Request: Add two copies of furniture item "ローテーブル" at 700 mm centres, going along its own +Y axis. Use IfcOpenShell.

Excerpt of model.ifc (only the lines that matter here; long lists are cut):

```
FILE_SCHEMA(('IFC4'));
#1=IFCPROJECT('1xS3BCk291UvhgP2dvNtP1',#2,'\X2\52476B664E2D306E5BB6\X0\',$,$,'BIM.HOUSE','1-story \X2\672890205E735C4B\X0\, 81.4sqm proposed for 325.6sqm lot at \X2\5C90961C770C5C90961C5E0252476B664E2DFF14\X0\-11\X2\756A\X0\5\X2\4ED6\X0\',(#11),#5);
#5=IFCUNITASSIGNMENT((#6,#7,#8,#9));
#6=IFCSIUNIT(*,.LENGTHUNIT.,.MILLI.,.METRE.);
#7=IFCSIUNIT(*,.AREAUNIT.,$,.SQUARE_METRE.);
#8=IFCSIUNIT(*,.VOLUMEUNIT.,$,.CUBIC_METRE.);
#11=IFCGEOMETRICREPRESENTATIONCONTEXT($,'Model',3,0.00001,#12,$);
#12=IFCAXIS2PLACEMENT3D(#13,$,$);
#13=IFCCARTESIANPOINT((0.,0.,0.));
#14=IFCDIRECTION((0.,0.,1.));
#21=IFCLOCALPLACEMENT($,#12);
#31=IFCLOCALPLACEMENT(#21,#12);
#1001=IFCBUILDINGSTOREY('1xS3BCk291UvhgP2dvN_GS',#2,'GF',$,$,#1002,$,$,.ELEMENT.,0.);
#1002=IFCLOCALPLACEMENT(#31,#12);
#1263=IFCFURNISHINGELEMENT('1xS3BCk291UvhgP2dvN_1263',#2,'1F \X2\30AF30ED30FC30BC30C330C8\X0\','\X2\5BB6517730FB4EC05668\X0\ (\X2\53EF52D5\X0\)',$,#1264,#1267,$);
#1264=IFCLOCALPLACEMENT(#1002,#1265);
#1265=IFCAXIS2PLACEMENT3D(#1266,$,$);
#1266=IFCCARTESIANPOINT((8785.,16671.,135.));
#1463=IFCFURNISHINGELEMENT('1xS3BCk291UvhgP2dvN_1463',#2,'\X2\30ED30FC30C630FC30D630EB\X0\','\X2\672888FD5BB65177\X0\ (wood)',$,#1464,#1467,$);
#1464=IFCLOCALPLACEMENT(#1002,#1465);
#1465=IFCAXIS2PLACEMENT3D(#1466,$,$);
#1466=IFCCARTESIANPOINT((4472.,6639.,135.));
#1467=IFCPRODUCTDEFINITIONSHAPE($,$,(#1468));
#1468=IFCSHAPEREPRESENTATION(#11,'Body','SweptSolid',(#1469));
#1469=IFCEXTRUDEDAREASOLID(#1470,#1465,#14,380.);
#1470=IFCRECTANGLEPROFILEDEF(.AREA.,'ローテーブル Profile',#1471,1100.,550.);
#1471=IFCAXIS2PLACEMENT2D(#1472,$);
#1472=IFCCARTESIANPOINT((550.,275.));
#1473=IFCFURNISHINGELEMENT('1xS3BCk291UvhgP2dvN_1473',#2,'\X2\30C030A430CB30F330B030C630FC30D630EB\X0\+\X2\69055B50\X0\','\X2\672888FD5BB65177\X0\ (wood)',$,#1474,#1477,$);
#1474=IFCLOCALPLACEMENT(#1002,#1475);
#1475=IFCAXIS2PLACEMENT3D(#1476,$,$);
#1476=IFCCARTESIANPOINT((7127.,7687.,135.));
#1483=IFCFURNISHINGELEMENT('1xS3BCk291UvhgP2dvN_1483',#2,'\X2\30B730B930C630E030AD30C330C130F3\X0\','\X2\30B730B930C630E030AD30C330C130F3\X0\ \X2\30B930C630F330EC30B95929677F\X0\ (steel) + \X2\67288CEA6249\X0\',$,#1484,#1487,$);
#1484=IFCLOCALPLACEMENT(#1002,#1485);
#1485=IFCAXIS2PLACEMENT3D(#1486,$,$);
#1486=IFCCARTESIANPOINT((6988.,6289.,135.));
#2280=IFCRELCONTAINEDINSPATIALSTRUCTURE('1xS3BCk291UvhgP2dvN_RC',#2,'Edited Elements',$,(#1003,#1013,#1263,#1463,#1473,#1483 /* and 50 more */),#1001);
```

```python
import ifcopenshell
import ifcopenshell.api.geometry
import ifcopenshell.api.root
import ifcopenshell.util.element
import ifcopenshell.util.placement
import ifcopenshell.util.unit

model = ifcopenshell.open("model.ifc")
unit_scale = ifcopenshell.util.unit.calculate_unit_scale(model)


def reuse_history(source, copy):
    """copy_class also copies each property set's owner history, people and application; keep the originals."""
    for rel in copy.IsDefinedBy:
        if rel.is_a("IfcRelDefinesByProperties") and (history := rel.RelatingPropertyDefinition.OwnerHistory):
            rel.RelatingPropertyDefinition.OwnerHistory = source.OwnerHistory
            ifcopenshell.util.element.remove_deep2(model, history)


source = model.by_id(1463)
base = ifcopenshell.util.placement.get_local_placement(source.ObjectPlacement)
step = base[:3, 1] * 0.7 / unit_scale

for i in range(1, 3):
    copy = ifcopenshell.api.root.copy_class(model, product=source)
    copy.Representation = ifcopenshell.util.element.copy_deep(
        model, source.Representation, exclude=["IfcGeometricRepresentationContext", "IfcRepresentationMap"]
    )
    reuse_history(source, copy)
    matrix = base.copy()
    matrix[:3, 3] += i * step
    print("added at", matrix[:3, 3].round(3) + 0.0)
    ifcopenshell.api.geometry.edit_object_placement(model, product=copy, matrix=matrix, is_si=False)

model.write("model_edited.ifc")
```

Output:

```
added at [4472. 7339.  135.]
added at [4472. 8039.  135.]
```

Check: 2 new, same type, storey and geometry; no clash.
